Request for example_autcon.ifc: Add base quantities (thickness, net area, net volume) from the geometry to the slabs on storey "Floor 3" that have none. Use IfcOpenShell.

First a look at what the model holds.

```python
import ifcopenshell
import ifcopenshell.util.element
import ifcopenshell.util.unit

model = ifcopenshell.open("example_autcon.ifc")
print(model.schema)
for unit_type in ("LENGTHUNIT", "AREAUNIT", "VOLUMEUNIT"):
    print(unit_type, ifcopenshell.util.unit.calculate_unit_scale(model, unit_type))
storey = next(s for s in model.by_type("IfcBuildingStorey") if s.Name == "Floor 3")
slabs = [e for e in ifcopenshell.util.element.get_decomposition(storey) if e.is_a("IfcSlab")]
for e in sorted(slabs, key=lambda e: e.id()):
    print(e.id(), e.is_a(), e.Name, list(ifcopenshell.util.element.get_psets(e, qtos_only=True)), sep=" | ")
```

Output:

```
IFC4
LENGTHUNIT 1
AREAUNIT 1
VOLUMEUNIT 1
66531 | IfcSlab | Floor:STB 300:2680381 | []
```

```python
import ifcopenshell
import ifcopenshell.api.pset
import ifcopenshell.geom
import ifcopenshell.util.element
import ifcopenshell.util.shape
import ifcopenshell.util.unit

model = ifcopenshell.open("example_autcon.ifc")
unit_scale = ifcopenshell.util.unit.calculate_unit_scale(model)
area_scale = ifcopenshell.util.unit.calculate_unit_scale(model, "AREAUNIT")
volume_scale = ifcopenshell.util.unit.calculate_unit_scale(model, "VOLUMEUNIT")
settings = ifcopenshell.geom.settings()

storey = next(s for s in model.by_type("IfcBuildingStorey") if s.Name == "Floor 3")
slabs = [e for e in ifcopenshell.util.element.get_decomposition(storey) if e.is_a("IfcSlab")]

for e in sorted(slabs, key=lambda e: e.id()):
    if ifcopenshell.util.element.get_psets(e, qtos_only=True, should_inherit=False):
        continue
    # Geometry comes back in metres, in the element's own axes.
    shape = ifcopenshell.geom.create_shape(settings, e)
    values = {
        "Width": ifcopenshell.util.shape.get_z(shape.geometry) / unit_scale,
        "NetArea": ifcopenshell.util.shape.get_footprint_area(shape.geometry) / area_scale,
        "NetVolume": ifcopenshell.util.shape.get_volume(shape.geometry) / volume_scale,
    }
    qto = ifcopenshell.api.pset.add_qto(model, product=e, name="Qto_SlabBaseQuantities")
    ifcopenshell.api.pset.edit_qto(model, qto=qto, properties=values)
    print(e.id(), {k: round(v, 3) for k, v in values.items()})

model.write("example_autcon_edited.ifc")
```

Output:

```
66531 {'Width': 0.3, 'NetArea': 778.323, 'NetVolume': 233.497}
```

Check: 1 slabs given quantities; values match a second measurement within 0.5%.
